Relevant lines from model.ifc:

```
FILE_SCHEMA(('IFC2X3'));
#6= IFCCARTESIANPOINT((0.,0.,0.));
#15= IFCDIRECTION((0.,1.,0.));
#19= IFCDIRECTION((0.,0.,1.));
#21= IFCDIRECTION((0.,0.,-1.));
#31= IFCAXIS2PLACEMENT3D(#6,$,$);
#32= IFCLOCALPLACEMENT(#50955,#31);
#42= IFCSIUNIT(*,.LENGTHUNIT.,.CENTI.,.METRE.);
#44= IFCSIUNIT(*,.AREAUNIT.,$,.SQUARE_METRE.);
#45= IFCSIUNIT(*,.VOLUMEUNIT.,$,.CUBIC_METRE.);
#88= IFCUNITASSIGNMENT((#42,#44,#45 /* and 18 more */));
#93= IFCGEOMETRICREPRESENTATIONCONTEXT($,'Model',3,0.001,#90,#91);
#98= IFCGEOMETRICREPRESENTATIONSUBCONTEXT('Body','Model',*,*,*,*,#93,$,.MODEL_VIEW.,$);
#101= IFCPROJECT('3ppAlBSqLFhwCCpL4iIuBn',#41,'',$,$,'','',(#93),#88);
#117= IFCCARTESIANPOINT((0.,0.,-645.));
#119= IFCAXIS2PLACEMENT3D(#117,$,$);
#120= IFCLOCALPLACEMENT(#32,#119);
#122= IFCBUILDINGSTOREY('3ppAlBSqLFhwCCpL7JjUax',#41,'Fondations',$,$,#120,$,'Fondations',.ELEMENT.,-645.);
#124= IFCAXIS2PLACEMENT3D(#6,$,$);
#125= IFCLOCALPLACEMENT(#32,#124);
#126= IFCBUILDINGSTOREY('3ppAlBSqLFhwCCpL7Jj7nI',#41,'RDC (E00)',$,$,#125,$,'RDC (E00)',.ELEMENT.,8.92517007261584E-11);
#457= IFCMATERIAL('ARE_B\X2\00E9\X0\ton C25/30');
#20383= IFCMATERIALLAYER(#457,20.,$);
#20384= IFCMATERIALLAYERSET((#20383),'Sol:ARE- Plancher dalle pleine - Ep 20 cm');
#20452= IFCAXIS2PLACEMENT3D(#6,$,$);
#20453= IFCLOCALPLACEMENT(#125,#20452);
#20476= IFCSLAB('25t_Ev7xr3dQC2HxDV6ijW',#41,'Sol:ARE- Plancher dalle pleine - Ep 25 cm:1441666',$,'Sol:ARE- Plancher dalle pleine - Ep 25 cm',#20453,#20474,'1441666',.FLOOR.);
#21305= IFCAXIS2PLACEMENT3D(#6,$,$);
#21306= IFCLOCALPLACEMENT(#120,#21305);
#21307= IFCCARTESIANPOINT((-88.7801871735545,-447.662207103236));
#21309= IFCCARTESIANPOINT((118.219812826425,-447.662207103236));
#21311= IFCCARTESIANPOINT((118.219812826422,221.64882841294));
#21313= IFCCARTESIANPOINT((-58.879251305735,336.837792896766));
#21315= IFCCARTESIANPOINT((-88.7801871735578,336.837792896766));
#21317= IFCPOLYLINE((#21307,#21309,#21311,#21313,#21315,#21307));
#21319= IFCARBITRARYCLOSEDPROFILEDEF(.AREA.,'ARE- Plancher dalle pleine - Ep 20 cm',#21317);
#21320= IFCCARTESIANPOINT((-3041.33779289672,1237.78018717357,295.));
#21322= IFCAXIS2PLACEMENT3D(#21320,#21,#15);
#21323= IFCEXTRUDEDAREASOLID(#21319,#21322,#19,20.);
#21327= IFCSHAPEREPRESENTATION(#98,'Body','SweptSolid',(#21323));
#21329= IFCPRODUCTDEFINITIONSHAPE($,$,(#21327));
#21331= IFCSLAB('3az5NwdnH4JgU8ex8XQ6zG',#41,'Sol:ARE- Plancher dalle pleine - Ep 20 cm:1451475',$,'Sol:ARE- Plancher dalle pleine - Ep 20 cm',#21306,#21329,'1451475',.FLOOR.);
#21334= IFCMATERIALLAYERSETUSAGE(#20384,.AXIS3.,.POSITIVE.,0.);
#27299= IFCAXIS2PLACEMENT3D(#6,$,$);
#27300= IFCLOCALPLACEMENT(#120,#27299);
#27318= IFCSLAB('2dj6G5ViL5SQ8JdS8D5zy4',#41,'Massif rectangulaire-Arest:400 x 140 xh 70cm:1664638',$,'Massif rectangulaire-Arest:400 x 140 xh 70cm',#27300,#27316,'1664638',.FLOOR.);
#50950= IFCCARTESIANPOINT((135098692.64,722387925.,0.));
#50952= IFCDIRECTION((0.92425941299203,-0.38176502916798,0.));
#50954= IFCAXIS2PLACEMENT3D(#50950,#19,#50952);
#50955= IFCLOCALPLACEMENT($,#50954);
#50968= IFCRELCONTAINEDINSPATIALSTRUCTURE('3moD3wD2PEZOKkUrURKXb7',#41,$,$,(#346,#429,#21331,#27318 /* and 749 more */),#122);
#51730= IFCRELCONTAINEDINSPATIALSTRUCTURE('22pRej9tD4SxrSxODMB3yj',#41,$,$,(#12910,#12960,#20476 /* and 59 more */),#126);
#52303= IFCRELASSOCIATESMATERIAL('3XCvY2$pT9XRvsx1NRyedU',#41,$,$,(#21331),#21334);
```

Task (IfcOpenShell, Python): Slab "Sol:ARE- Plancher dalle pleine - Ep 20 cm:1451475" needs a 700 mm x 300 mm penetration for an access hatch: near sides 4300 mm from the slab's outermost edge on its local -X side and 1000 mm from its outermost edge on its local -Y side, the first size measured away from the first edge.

```python
import numpy as np
import ifcopenshell
import ifcopenshell.api.feature
import ifcopenshell.api.geometry
import ifcopenshell.api.root
import ifcopenshell.geom
import ifcopenshell.util.placement
import ifcopenshell.util.representation
import ifcopenshell.util.shape
import ifcopenshell.util.unit

model = ifcopenshell.open("model.ifc")
unit_scale = ifcopenshell.util.unit.calculate_unit_scale(model)
settings = ifcopenshell.geom.settings()


def volume(element):
    """Net volume in cubic metres, openings subtracted."""
    shape = ifcopenshell.geom.create_shape(settings, element)
    return ifcopenshell.util.shape.get_volume(shape.geometry)


slab = model.by_id(21331)
before = volume(slab)

# Extent in the slab's own axes, in metres. The edges named are its -X and -Y sides.
slab_shape = ifcopenshell.geom.create_shape(settings, slab)
vertices = ifcopenshell.util.shape.get_vertices(slab_shape.geometry)
x_min, y_min, bottom = vertices.min(axis=0)
top = vertices[:, 2].max()

opening = ifcopenshell.api.root.create_entity(model, ifc_class="IfcOpeningElement", name="Access hatch opening")
context = ifcopenshell.util.representation.get_context(model, "Model", "Body", "MODEL_VIEW")
width, depth = 0.7, 0.3
outline = [(0.0, 0.0), (width, 0.0), (width, depth), (0.0, depth), (0.0, 0.0)]
# Overshoot both faces by 50 mm so the cut is clean.
shape = ifcopenshell.api.geometry.add_slab_representation(
    model, context=context, depth=top - bottom + 0.1, polyline=outline
)
ifcopenshell.api.geometry.assign_representation(model, product=opening, representation=shape)

matrix = ifcopenshell.util.placement.get_local_placement(slab.ObjectPlacement)
matrix[:, 3] = matrix @ np.append(np.array([x_min + 4.3, y_min + 1, bottom - 0.05]) / unit_scale, 1.0)
ifcopenshell.api.geometry.edit_object_placement(model, product=opening, matrix=matrix, is_si=False)
ifcopenshell.api.feature.add_feature(model, feature=opening, element=slab)

after = volume(slab)

print(f"slab volume {before:.3f} -> {after:.3f} m3")

model.write("model_edited.ifc")
```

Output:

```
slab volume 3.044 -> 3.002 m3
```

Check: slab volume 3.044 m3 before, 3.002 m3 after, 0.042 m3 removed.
